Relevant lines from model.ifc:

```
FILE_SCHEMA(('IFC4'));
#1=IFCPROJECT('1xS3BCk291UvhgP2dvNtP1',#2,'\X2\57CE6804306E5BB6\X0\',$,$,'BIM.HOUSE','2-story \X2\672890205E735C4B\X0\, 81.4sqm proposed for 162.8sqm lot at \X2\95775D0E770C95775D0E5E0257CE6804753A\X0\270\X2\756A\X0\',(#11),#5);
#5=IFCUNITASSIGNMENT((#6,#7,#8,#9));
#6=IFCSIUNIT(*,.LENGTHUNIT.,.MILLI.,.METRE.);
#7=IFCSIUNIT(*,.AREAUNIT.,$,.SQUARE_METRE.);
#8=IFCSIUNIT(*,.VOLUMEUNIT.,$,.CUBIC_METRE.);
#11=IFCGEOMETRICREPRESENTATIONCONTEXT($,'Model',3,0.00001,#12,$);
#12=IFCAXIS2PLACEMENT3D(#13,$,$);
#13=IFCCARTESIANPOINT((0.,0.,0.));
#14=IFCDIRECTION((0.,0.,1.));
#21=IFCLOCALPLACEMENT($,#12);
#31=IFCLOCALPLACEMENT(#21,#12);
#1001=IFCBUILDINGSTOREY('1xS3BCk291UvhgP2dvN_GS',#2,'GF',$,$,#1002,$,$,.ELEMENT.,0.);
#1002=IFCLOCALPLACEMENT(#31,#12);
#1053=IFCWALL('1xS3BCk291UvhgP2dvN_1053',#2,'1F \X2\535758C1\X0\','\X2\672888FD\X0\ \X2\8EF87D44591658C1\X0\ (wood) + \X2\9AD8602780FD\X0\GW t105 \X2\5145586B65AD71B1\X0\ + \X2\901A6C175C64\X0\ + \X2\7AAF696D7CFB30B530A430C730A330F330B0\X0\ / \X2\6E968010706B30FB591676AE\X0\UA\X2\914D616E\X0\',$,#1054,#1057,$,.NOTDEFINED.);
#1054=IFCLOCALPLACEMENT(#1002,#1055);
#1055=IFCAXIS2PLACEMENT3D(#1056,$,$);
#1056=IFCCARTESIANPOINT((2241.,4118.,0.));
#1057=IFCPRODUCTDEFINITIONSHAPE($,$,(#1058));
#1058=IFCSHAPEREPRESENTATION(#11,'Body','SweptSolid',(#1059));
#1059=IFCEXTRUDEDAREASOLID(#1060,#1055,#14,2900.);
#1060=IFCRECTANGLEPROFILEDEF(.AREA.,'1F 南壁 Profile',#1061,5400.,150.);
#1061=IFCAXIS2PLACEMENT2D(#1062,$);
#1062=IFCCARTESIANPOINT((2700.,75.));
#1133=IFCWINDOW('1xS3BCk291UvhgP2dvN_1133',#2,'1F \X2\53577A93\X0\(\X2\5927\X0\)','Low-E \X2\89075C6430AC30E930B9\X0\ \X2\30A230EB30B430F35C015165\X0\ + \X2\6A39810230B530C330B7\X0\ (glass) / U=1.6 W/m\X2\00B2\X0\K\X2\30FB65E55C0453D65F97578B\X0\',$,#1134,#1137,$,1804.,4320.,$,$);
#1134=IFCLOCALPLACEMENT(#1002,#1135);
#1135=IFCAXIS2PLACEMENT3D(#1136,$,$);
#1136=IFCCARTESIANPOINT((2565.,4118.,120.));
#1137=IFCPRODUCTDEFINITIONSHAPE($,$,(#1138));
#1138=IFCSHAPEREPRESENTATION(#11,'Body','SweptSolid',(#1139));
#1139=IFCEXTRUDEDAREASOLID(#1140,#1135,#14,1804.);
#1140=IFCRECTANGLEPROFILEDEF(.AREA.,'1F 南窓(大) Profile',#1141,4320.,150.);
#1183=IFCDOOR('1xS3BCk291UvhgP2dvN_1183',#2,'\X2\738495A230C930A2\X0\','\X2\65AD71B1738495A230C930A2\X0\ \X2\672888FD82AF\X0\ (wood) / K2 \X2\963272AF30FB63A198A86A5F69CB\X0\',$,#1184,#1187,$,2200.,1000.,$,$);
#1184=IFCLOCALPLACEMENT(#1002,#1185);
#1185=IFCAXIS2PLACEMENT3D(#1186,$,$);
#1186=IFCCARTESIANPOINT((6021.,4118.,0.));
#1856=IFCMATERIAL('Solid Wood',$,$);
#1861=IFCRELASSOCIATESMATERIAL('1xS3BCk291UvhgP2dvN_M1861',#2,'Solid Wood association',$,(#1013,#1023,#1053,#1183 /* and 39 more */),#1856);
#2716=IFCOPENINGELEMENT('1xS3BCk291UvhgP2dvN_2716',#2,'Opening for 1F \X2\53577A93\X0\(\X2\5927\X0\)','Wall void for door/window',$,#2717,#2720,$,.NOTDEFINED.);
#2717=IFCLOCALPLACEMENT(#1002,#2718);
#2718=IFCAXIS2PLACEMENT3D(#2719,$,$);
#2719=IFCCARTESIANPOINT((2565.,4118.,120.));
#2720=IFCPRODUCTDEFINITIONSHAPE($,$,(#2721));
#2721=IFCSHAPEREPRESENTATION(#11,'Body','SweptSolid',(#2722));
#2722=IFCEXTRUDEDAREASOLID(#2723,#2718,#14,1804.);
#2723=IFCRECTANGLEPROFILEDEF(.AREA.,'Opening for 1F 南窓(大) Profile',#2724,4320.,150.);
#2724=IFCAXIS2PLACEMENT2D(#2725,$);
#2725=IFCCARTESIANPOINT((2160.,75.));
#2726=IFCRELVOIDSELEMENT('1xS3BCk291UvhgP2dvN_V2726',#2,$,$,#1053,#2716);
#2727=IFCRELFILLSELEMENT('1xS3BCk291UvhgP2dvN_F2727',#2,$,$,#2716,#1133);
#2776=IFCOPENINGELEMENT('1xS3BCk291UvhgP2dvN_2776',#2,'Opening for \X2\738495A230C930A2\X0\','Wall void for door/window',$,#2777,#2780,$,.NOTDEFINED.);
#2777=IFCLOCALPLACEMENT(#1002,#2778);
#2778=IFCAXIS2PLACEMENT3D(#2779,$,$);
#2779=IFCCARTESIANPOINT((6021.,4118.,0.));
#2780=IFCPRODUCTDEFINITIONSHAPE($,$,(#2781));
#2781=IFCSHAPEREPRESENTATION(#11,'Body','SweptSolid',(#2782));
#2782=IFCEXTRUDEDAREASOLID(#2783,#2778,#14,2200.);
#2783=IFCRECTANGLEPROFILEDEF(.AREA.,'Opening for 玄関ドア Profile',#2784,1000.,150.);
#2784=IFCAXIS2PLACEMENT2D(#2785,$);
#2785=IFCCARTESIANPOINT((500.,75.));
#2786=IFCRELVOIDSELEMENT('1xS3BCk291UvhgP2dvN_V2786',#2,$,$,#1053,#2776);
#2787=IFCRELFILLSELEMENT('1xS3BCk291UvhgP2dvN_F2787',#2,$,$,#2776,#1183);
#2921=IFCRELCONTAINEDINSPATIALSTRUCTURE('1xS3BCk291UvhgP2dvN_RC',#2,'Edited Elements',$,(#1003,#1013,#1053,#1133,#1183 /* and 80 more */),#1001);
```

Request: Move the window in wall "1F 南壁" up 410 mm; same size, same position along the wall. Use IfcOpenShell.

```python
import numpy as np
import ifcopenshell
import ifcopenshell.api.geometry
import ifcopenshell.util.placement
import ifcopenshell.util.unit

model = ifcopenshell.open("model.ifc")
unit_scale = ifcopenshell.util.unit.calculate_unit_scale(model)

window = model.by_guid("1xS3BCk291UvhgP2dvN_1133")
opening = window.FillsVoids[0].RelatingOpeningElement
dz = 410.0

shift = np.array([0.0, 0.0, dz])
# The window is not placed relative to its opening, so move both.
for product in (opening, window):
    matrix = ifcopenshell.util.placement.get_local_placement(product.ObjectPlacement)
    matrix[:3, 3] += shift
    ifcopenshell.api.geometry.edit_object_placement(model, product=product, matrix=matrix, is_si=False)

print(f"moved by {dz * unit_scale:+.3f} m")

model.write("model_edited.ifc")
```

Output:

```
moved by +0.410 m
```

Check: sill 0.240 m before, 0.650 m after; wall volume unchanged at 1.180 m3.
